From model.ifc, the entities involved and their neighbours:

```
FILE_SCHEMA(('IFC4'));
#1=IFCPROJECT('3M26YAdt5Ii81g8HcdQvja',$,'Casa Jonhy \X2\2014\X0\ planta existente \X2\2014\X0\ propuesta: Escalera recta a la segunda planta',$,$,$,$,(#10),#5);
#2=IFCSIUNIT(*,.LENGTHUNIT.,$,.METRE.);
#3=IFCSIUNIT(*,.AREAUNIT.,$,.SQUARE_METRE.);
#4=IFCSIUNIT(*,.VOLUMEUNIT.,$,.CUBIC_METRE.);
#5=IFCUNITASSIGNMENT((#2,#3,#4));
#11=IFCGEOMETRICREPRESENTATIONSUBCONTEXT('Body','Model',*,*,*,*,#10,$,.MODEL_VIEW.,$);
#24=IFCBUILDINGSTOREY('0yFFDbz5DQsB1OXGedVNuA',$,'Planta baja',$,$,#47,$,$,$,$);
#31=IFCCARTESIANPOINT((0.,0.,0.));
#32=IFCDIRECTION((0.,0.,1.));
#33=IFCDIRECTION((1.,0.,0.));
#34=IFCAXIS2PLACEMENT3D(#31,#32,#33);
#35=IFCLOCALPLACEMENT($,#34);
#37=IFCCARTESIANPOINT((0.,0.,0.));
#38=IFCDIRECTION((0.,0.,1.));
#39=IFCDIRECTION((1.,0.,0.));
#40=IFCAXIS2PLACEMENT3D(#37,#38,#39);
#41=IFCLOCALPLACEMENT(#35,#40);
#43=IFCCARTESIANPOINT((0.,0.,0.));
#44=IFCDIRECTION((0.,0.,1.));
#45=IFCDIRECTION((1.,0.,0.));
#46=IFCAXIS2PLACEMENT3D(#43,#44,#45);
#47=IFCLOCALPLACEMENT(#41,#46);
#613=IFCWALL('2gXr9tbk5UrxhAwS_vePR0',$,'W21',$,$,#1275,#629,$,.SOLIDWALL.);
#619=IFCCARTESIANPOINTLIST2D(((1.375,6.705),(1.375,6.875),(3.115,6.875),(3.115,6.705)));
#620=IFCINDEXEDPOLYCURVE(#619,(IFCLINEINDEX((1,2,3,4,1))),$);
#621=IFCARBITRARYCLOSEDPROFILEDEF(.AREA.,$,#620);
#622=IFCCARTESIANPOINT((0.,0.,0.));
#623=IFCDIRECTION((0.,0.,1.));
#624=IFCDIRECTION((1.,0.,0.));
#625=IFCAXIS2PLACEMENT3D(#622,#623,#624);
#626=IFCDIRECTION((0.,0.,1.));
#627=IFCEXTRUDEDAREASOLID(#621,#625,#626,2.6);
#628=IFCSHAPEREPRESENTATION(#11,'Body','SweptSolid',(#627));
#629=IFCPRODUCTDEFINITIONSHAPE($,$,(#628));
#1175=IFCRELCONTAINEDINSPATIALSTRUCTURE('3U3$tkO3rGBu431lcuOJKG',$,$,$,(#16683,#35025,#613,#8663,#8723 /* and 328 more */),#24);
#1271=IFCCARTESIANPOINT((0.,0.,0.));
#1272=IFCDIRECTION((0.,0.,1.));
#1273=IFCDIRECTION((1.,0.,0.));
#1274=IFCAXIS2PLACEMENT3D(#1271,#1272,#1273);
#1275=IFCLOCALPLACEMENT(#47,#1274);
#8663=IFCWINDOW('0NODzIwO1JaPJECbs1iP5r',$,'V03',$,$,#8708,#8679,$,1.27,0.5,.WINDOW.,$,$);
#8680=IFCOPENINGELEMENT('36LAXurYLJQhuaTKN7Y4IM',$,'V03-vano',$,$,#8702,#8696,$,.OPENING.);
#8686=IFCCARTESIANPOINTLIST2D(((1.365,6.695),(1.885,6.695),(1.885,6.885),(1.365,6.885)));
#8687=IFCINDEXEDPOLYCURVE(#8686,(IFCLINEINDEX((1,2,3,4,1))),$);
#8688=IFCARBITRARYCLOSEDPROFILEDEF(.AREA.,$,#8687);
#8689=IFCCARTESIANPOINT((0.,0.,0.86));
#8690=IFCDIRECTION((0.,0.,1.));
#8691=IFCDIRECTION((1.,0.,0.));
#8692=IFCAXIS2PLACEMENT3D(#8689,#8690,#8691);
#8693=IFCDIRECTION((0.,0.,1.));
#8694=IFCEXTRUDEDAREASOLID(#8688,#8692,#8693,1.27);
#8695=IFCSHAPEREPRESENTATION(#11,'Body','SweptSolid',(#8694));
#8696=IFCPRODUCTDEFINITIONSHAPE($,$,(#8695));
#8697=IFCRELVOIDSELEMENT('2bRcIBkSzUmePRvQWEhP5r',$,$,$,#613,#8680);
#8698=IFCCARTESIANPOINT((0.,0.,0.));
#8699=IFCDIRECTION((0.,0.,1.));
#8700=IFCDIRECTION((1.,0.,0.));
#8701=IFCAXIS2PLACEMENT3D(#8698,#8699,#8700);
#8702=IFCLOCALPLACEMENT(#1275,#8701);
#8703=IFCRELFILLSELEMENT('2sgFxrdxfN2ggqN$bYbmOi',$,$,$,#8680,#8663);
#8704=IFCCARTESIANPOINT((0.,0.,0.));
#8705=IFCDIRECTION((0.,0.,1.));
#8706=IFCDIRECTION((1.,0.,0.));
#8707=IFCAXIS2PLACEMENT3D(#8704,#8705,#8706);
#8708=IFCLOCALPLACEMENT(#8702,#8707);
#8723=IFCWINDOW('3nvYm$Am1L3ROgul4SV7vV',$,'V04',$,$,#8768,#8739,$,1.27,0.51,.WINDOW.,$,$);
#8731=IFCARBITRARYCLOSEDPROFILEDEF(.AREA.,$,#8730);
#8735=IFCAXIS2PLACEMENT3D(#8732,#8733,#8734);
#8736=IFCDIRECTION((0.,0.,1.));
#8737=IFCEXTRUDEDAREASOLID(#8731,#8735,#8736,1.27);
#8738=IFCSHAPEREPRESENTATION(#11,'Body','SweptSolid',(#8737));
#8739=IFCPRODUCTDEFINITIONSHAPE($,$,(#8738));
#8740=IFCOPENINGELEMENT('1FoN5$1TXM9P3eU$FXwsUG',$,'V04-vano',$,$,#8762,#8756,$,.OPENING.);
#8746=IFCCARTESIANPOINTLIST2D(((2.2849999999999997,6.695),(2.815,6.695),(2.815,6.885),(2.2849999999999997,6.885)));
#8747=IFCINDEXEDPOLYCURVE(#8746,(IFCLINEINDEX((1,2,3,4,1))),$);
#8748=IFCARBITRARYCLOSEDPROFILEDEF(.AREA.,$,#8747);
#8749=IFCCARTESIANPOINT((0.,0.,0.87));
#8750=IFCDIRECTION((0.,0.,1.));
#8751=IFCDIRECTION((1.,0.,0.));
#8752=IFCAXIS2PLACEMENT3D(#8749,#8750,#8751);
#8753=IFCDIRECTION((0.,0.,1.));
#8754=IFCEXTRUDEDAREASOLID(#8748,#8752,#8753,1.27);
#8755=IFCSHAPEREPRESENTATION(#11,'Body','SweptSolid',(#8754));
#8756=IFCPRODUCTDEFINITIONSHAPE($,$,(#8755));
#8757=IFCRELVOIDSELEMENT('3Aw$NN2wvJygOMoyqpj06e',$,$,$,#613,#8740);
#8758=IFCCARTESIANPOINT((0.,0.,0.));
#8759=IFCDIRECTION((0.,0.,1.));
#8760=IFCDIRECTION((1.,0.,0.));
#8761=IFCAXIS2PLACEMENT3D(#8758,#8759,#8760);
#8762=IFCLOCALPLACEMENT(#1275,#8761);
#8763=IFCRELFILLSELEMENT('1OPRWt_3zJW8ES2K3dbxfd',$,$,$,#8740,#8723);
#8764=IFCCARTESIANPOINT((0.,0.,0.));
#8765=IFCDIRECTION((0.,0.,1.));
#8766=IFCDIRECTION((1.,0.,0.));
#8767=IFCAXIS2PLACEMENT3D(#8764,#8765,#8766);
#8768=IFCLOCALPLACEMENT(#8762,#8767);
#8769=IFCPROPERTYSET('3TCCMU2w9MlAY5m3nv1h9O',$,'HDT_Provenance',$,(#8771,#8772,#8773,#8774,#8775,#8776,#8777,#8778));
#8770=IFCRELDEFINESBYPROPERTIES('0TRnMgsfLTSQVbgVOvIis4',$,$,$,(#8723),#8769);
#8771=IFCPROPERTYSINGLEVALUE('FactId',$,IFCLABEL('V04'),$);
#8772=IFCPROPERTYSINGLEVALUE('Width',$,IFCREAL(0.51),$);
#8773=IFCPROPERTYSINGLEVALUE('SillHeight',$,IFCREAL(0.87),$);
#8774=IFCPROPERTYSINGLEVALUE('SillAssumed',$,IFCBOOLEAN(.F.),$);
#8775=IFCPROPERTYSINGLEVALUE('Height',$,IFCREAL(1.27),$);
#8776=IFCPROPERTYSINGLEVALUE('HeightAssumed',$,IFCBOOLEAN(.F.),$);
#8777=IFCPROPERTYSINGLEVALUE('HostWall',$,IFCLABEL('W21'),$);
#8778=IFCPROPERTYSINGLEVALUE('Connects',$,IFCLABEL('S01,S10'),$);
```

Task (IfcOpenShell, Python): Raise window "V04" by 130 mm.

```python
import numpy as np
import ifcopenshell
import ifcopenshell.api.geometry
import ifcopenshell.api.pset
import ifcopenshell.util.element
import ifcopenshell.util.placement
import ifcopenshell.util.unit

model = ifcopenshell.open("model.ifc")
unit_scale = ifcopenshell.util.unit.calculate_unit_scale(model)

window = model.by_guid("3nvYm$Am1L3ROgul4SV7vV")
opening = window.FillsVoids[0].RelatingOpeningElement
dz = 0.13 / unit_scale

shift = np.array([0.0, 0.0, dz])
# The window is placed relative to its opening, so it follows when the opening moves.
matrix = ifcopenshell.util.placement.get_local_placement(opening.ObjectPlacement)
matrix[:3, 3] += shift
ifcopenshell.api.geometry.edit_object_placement(
    model, product=opening, matrix=matrix, is_si=False, should_transform_children=True
)

# Keep the stored heights in step.
pset = model.by_id(ifcopenshell.util.element.get_pset(window, "HDT_Provenance", should_inherit=False)["id"])
ifcopenshell.api.pset.edit_pset(model, pset=pset, properties={
    "SillHeight": model.create_entity("IfcReal", ifcopenshell.util.element.get_pset(window, "HDT_Provenance", "SillHeight") + dz),
})

print(f"moved by {dz * unit_scale:+.3f} m")

model.write("model_updated.ifc")
```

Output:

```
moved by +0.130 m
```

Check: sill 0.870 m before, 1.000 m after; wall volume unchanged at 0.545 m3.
